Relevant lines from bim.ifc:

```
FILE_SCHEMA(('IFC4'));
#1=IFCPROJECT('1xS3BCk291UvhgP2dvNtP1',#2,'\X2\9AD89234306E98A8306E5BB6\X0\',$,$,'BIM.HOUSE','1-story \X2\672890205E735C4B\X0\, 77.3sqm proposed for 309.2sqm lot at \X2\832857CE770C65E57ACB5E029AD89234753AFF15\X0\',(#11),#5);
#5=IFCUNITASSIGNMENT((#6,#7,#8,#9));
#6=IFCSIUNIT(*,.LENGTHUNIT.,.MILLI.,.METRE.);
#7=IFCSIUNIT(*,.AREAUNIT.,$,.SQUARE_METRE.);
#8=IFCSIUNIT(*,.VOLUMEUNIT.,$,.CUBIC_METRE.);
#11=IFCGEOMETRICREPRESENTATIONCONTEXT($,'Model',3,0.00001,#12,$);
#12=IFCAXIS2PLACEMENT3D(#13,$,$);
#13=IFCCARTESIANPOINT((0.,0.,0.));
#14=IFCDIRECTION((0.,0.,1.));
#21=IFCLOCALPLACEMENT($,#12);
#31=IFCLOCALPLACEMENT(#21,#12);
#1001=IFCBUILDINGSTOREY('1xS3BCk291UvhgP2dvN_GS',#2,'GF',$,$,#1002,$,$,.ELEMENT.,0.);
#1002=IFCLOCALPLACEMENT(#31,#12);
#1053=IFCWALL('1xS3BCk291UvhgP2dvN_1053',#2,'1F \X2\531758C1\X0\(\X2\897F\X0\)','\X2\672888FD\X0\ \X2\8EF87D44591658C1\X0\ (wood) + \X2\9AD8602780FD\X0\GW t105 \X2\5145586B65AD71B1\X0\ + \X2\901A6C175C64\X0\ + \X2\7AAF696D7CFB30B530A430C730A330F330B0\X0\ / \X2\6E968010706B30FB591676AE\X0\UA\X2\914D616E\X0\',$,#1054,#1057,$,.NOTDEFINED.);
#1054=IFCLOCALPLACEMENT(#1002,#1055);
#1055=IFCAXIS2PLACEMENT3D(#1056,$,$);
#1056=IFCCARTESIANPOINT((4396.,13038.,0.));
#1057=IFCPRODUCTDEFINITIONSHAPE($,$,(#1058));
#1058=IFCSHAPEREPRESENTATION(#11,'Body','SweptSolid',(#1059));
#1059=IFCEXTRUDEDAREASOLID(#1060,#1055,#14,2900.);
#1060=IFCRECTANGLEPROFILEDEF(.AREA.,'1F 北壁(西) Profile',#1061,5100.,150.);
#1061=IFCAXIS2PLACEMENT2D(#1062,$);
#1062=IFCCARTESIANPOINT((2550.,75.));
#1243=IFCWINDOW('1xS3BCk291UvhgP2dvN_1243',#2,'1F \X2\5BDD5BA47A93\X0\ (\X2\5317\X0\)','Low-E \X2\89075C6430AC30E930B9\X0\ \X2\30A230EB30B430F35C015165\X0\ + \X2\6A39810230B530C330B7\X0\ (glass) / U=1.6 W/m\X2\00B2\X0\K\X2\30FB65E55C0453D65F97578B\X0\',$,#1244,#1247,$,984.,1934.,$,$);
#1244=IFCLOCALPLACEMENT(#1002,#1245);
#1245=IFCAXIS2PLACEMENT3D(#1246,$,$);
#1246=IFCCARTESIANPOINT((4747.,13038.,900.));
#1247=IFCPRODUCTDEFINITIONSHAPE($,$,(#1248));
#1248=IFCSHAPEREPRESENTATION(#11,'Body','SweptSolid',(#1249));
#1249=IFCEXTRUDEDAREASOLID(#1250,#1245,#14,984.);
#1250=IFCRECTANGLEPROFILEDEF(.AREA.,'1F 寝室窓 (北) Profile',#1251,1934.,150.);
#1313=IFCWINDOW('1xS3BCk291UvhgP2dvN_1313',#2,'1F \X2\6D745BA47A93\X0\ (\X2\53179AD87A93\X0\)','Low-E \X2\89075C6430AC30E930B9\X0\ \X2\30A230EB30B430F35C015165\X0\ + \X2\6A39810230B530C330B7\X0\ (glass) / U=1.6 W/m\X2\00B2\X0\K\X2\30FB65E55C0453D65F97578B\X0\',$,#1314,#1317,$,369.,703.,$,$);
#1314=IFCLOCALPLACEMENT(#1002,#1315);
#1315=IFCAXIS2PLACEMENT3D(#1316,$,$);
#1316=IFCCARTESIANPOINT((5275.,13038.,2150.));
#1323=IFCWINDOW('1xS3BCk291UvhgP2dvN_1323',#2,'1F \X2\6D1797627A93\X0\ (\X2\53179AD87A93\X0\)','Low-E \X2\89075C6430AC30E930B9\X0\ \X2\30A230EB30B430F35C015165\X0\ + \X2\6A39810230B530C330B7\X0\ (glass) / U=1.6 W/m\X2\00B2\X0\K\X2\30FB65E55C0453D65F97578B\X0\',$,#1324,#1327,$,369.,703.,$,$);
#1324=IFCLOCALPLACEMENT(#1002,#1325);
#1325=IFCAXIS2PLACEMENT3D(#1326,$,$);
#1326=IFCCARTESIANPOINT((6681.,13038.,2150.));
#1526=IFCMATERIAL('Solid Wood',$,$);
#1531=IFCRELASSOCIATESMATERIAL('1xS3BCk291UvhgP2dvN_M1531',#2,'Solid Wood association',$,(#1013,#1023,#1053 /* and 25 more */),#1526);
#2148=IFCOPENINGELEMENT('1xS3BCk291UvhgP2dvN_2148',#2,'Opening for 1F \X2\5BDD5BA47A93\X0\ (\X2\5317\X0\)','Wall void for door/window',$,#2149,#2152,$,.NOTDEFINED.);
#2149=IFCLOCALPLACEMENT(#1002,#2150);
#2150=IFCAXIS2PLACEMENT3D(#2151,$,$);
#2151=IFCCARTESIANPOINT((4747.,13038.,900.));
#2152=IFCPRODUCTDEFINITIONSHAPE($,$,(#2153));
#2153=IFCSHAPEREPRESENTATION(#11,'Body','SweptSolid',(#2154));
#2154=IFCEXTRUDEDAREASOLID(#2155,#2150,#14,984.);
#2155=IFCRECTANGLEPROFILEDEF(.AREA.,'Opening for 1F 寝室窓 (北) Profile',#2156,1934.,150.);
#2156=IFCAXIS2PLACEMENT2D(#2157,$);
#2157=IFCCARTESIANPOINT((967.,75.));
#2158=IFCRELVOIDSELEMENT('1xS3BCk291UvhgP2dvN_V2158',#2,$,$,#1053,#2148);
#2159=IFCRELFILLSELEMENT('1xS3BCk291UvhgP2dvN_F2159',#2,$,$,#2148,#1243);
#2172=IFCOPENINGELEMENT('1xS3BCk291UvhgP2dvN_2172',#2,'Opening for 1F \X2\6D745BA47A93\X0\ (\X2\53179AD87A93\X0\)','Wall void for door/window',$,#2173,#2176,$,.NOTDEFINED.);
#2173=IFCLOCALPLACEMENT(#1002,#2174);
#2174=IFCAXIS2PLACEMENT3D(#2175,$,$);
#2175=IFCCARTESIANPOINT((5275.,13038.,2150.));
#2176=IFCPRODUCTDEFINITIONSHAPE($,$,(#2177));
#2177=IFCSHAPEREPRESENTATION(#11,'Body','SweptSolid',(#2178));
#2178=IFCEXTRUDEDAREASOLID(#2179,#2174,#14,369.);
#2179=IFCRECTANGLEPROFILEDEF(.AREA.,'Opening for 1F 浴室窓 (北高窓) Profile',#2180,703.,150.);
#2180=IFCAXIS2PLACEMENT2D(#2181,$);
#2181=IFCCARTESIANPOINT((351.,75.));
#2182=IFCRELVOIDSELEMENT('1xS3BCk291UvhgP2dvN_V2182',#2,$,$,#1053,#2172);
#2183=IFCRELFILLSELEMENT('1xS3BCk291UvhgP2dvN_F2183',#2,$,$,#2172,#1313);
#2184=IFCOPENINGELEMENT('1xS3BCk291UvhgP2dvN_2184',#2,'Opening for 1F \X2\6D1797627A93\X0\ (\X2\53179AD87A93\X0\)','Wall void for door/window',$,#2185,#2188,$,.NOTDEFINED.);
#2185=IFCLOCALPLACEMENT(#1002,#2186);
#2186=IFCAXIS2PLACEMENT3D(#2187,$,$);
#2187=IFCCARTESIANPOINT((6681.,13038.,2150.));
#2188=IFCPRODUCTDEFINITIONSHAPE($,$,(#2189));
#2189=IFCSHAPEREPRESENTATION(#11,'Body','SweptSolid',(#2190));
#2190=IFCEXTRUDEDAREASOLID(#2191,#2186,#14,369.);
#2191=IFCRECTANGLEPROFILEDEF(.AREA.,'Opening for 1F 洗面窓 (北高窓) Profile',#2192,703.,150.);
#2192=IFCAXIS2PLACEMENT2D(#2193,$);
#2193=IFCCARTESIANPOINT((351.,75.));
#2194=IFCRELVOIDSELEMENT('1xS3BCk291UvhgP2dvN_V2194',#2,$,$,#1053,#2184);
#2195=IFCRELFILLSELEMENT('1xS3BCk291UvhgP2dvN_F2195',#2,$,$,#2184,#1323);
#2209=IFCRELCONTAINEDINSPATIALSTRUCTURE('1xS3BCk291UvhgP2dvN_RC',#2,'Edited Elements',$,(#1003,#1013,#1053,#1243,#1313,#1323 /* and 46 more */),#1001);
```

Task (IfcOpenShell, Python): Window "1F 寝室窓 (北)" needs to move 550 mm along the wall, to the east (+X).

```python
import ifcopenshell
import ifcopenshell.api.geometry
import ifcopenshell.util.placement
import ifcopenshell.util.unit

model = ifcopenshell.open("bim.ifc")
unit_scale = ifcopenshell.util.unit.calculate_unit_scale(model)

window = model.by_id(1243)
opening = window.FillsVoids[0].RelatingOpeningElement
wall = opening.VoidsElements[0].RelatingBuildingElement

wall_matrix = ifcopenshell.util.placement.get_local_placement(wall.ObjectPlacement)
shift = wall_matrix[:3, 0] * 0.55 / unit_scale
before = ifcopenshell.util.placement.get_local_placement(window.ObjectPlacement)[:3, 3].copy()

# The window is not placed relative to its opening, so move both.
for product in (opening, window):
    matrix = ifcopenshell.util.placement.get_local_placement(product.ObjectPlacement)
    matrix[:3, 3] += shift
    ifcopenshell.api.geometry.edit_object_placement(model, product=product, matrix=matrix, is_si=False)

after = ifcopenshell.util.placement.get_local_placement(window.ObjectPlacement)[:3, 3]
print("window moved by", (after - before).round(3) + 0.0)

model.write("bim_edited.ifc")
```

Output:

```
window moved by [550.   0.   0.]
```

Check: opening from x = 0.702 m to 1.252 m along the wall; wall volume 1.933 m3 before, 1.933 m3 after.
